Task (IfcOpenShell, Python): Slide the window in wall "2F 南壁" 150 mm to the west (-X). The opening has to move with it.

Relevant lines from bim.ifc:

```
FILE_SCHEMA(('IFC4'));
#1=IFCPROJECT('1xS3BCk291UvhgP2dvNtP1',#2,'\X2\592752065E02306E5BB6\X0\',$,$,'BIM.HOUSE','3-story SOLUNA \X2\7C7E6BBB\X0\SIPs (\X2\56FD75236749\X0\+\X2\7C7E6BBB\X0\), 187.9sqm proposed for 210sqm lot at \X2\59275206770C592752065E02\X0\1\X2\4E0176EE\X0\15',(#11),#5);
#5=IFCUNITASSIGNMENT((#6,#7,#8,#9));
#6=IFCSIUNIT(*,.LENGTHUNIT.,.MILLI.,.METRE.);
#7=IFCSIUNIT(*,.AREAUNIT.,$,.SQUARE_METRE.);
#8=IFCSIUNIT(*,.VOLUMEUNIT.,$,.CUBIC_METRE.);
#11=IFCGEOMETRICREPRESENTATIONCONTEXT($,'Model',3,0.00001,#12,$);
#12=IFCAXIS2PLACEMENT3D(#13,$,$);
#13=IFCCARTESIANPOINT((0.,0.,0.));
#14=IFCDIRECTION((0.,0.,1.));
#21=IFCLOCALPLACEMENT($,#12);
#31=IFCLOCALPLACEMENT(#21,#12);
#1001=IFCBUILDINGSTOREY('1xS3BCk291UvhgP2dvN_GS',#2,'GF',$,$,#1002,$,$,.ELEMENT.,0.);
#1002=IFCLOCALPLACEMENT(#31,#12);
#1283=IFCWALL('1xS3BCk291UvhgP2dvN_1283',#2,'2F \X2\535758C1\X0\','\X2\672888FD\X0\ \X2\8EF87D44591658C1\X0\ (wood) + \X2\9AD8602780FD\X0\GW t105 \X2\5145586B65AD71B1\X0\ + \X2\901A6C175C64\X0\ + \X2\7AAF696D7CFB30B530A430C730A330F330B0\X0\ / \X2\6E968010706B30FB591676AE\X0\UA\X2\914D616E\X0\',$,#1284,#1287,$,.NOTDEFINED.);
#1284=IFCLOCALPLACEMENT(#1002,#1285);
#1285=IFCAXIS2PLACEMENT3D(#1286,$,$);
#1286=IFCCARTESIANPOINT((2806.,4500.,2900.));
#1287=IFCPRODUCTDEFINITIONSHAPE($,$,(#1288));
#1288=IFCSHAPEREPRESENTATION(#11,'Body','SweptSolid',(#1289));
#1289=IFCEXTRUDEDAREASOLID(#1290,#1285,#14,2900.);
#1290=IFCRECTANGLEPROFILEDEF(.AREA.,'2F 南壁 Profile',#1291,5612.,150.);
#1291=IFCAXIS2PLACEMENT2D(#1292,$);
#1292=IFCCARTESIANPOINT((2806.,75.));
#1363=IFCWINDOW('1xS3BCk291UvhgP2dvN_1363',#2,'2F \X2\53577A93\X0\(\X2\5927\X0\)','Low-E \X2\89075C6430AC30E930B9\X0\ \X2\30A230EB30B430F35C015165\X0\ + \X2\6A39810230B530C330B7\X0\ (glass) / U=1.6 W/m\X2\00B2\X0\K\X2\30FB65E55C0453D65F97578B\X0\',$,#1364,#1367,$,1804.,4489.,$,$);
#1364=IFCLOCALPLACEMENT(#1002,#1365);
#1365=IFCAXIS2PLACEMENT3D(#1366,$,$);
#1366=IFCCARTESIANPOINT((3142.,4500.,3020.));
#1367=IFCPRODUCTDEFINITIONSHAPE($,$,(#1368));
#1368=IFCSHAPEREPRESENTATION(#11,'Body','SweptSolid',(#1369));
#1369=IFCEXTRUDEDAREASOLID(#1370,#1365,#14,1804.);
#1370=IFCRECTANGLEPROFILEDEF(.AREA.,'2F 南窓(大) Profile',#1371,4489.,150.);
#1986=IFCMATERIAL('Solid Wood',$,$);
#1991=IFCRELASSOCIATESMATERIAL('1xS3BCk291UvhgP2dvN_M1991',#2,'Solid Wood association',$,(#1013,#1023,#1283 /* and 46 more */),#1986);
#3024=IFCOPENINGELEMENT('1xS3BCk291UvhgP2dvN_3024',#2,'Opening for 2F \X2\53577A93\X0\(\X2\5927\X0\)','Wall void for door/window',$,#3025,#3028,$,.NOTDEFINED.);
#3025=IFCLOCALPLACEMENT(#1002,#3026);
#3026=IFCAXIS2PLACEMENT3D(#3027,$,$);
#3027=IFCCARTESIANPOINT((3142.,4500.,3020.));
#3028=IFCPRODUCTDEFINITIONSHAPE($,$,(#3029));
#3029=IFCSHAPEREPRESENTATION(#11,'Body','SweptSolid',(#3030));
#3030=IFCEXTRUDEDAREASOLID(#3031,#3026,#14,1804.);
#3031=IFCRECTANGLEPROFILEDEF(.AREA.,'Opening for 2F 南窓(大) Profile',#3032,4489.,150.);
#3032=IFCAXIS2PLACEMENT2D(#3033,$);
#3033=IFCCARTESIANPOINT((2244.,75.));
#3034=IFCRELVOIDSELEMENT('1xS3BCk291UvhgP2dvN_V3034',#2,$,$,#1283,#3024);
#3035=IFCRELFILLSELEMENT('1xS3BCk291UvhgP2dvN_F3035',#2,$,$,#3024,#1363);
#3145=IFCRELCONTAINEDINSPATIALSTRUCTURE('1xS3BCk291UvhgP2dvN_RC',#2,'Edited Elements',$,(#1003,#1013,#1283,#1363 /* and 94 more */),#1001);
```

```python
import ifcopenshell
import ifcopenshell.api.geometry
import ifcopenshell.util.placement
import ifcopenshell.util.unit

model = ifcopenshell.open("bim.ifc")
unit_scale = ifcopenshell.util.unit.calculate_unit_scale(model)

window = model.by_id(1363)
opening = window.FillsVoids[0].RelatingOpeningElement
wall = opening.VoidsElements[0].RelatingBuildingElement

wall_matrix = ifcopenshell.util.placement.get_local_placement(wall.ObjectPlacement)
shift = wall_matrix[:3, 0] * -0.15 / unit_scale
before = ifcopenshell.util.placement.get_local_placement(window.ObjectPlacement)[:3, 3].copy()

# The window is not placed relative to its opening, so move both.
for product in (opening, window):
    matrix = ifcopenshell.util.placement.get_local_placement(product.ObjectPlacement)
    matrix[:3, 3] += shift
    ifcopenshell.api.geometry.edit_object_placement(model, product=product, matrix=matrix, is_si=False)

after = ifcopenshell.util.placement.get_local_placement(window.ObjectPlacement)[:3, 3]
print("window moved by", (after - before).round(3) + 0.0)

model.write("bim_v2.ifc")
```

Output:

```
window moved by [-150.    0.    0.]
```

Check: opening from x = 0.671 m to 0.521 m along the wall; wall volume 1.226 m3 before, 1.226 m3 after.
